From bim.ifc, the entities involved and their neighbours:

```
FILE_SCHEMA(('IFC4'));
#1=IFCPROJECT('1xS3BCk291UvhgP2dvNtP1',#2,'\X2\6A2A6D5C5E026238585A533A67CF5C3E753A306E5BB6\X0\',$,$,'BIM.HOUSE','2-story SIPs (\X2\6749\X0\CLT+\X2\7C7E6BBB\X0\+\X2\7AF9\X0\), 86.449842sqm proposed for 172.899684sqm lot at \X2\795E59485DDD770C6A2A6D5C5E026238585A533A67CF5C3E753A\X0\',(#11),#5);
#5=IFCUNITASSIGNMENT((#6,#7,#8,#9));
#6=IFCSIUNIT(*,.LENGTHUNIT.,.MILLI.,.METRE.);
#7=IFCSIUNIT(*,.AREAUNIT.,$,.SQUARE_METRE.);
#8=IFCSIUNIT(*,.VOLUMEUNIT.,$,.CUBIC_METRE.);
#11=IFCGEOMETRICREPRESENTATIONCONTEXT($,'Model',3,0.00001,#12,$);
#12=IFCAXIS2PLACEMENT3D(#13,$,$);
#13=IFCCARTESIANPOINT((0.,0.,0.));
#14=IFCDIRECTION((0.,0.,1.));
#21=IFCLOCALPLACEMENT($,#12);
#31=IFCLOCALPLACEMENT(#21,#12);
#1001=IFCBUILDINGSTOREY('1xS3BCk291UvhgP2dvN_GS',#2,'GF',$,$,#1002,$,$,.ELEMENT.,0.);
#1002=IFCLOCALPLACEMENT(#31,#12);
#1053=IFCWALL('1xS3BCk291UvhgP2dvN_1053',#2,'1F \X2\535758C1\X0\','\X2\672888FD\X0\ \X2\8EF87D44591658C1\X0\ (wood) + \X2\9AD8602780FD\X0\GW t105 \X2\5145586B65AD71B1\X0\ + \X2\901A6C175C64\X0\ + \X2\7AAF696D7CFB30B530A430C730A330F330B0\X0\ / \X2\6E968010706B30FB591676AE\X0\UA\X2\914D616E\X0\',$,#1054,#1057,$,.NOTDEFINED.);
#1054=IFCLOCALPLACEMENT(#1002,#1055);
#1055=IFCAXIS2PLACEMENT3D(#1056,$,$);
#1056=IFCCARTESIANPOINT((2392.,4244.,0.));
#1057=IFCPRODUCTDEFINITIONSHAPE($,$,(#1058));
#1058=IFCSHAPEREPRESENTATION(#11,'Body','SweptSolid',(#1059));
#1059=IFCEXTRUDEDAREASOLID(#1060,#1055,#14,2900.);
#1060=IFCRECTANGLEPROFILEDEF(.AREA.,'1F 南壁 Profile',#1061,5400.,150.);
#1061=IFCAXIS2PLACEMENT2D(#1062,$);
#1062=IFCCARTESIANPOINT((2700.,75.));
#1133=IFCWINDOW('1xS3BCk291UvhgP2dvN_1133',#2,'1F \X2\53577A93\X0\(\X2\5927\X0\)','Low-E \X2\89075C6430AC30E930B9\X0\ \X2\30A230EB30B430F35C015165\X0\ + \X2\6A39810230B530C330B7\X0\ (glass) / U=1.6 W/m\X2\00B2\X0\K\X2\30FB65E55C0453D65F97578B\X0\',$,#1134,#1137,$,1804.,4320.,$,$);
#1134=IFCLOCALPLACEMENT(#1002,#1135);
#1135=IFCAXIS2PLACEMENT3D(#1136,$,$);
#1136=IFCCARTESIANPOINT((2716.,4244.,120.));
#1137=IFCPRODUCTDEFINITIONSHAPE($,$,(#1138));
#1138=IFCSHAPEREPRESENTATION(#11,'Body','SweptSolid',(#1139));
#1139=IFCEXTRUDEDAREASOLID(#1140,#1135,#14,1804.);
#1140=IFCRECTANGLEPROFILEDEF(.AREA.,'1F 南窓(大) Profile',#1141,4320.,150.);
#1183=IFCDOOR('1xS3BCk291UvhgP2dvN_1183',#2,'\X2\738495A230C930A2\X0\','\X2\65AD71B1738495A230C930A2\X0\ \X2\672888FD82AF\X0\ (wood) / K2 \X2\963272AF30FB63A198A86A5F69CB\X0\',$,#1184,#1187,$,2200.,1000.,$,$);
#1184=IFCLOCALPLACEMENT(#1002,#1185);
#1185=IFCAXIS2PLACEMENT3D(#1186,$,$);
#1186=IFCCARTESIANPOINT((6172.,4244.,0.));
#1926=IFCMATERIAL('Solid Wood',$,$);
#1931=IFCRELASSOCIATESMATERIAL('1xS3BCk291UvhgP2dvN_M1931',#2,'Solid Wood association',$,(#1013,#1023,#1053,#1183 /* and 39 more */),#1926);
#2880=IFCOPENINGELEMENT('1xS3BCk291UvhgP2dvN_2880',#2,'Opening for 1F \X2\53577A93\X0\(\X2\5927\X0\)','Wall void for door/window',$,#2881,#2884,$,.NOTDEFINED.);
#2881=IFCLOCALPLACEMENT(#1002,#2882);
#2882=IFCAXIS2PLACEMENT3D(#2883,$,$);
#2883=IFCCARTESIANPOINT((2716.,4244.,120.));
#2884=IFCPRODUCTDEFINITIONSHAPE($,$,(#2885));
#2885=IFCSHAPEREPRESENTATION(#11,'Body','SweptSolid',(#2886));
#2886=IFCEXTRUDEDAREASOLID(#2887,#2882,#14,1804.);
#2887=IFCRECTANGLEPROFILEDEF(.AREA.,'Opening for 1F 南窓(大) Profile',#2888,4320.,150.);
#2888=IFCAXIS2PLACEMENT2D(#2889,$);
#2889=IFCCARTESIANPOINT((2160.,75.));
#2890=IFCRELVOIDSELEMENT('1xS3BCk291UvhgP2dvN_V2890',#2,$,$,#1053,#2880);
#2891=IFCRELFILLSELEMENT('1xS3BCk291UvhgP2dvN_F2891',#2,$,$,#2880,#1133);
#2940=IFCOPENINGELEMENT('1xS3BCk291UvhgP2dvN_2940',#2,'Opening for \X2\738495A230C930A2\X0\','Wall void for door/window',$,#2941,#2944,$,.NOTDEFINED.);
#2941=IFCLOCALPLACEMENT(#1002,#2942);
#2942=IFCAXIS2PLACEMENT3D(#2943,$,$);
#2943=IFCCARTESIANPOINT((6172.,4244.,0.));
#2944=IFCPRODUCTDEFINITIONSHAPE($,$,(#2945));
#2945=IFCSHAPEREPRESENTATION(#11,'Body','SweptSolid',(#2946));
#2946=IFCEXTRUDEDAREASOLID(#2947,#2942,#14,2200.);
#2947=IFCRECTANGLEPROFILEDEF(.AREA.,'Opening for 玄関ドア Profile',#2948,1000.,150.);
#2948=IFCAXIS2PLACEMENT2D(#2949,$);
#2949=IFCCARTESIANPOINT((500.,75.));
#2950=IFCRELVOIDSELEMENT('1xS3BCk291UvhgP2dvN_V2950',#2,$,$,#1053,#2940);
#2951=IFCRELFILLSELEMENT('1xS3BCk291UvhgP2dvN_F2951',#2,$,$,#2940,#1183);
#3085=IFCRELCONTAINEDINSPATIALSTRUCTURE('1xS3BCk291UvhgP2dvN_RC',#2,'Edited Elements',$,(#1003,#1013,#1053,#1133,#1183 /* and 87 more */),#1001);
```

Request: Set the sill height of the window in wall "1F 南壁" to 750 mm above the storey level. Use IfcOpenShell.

```python
import numpy as np
import ifcopenshell
import ifcopenshell.api.geometry
import ifcopenshell.geom
import ifcopenshell.util.element
import ifcopenshell.util.placement
import ifcopenshell.util.shape
import ifcopenshell.util.unit

model = ifcopenshell.open("bim.ifc")
unit_scale = ifcopenshell.util.unit.calculate_unit_scale(model)

window = model.by_guid("1xS3BCk291UvhgP2dvN_1133")
opening = window.FillsVoids[0].RelatingOpeningElement
storey = ifcopenshell.util.element.get_container(window, ifc_class="IfcBuildingStorey")
level = ifcopenshell.util.placement.get_local_placement(storey.ObjectPlacement)[2, 3]

# The opening's origin need not be at the sill, so measure its lowest point.
shape = ifcopenshell.geom.create_shape(ifcopenshell.geom.settings(), opening)
bottom = ifcopenshell.util.shape.get_shape_bottom_elevation(shape, shape.geometry) / unit_scale
dz = level + 0.75 / unit_scale - bottom

shift = np.array([0.0, 0.0, dz])
# The window is not placed relative to its opening, so move both.
for product in (opening, window):
    matrix = ifcopenshell.util.placement.get_local_placement(product.ObjectPlacement)
    matrix[:3, 3] += shift
    ifcopenshell.api.geometry.edit_object_placement(model, product=product, matrix=matrix, is_si=False)

print(f"moved by {dz * unit_scale:+.3f} m")

model.write("bim_updated.ifc")
```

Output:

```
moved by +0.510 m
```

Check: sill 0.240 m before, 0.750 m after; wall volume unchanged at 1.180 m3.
